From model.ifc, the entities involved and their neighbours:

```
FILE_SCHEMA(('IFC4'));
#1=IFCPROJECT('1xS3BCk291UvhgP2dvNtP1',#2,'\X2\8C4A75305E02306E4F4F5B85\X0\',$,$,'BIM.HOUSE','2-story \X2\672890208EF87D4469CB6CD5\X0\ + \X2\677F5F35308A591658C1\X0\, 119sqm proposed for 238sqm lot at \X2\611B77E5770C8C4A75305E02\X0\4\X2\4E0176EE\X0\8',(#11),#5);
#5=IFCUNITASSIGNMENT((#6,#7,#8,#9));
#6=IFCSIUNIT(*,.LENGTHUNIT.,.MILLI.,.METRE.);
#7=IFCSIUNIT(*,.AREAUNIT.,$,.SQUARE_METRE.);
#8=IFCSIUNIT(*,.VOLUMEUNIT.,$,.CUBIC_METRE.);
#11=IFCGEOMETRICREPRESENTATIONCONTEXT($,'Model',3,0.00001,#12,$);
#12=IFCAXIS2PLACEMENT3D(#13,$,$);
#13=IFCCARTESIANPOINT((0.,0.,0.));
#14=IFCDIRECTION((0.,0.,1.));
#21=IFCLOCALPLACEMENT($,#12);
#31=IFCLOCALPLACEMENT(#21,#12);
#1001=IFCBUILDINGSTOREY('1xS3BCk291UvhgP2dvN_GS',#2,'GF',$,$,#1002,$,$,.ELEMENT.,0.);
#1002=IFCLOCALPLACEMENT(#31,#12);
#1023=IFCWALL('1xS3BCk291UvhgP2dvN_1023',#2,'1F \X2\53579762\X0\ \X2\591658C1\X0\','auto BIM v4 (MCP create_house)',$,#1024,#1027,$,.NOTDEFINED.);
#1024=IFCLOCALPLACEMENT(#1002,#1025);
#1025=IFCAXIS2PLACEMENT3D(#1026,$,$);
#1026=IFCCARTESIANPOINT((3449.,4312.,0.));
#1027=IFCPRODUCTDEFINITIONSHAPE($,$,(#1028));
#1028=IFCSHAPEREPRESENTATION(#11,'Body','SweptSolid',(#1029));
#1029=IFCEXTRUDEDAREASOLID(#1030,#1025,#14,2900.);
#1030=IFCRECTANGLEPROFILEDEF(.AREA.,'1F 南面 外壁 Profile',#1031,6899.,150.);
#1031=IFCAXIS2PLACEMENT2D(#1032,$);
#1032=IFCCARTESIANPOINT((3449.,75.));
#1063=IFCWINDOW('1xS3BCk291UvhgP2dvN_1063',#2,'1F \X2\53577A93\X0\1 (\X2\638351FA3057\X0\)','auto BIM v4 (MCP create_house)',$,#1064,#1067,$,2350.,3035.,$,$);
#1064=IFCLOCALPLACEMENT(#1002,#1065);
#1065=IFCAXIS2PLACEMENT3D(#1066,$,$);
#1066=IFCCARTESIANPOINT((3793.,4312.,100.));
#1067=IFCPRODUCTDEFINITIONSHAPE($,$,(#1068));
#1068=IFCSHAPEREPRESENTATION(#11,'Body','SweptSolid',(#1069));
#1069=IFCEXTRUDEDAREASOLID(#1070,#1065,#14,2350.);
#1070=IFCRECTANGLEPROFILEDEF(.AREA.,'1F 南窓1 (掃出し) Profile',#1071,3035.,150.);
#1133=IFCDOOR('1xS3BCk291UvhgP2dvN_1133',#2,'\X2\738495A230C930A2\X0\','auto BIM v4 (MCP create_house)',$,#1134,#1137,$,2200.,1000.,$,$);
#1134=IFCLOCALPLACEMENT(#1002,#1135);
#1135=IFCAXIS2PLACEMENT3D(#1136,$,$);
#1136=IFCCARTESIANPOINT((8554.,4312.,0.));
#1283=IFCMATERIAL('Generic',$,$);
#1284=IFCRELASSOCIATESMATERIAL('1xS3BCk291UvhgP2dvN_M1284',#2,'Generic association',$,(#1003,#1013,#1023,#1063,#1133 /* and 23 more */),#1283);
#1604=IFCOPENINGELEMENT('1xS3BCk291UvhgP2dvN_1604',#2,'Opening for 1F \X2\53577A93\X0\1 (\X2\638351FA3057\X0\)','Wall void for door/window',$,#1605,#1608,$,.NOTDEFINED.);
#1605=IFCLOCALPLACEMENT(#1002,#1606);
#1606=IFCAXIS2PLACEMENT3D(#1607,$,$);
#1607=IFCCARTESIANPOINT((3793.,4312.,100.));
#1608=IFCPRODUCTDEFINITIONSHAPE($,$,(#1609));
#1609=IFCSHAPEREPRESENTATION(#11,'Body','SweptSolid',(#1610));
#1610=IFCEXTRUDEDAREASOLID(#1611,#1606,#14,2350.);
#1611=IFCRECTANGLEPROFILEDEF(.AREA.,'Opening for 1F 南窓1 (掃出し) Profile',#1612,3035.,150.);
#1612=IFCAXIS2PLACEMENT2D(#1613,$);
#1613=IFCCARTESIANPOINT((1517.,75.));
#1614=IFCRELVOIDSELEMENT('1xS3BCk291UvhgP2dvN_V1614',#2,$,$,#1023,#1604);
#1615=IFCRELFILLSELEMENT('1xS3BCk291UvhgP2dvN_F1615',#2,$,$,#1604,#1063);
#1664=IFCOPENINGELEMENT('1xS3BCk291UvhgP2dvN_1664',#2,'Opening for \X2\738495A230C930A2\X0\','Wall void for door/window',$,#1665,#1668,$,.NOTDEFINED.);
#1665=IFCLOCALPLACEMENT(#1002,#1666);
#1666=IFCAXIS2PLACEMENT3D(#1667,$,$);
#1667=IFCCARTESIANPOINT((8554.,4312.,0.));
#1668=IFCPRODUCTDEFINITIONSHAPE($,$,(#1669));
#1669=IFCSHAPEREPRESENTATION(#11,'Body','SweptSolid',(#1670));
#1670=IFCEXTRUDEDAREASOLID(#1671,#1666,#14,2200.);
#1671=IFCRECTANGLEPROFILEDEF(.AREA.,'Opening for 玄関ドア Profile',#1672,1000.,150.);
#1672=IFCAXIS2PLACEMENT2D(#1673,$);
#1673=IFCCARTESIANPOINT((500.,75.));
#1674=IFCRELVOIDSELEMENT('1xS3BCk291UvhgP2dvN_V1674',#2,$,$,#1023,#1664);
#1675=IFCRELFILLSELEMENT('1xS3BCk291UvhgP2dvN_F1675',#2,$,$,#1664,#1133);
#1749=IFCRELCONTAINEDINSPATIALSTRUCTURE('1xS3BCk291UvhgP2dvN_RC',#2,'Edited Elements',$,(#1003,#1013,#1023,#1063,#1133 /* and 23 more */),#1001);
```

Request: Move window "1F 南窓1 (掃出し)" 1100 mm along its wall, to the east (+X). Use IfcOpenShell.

```python
import ifcopenshell
import ifcopenshell.api.geometry
import ifcopenshell.util.placement
import ifcopenshell.util.unit

model = ifcopenshell.open("model.ifc")
unit_scale = ifcopenshell.util.unit.calculate_unit_scale(model)

window = model.by_id(1063)
opening = window.FillsVoids[0].RelatingOpeningElement
wall = opening.VoidsElements[0].RelatingBuildingElement

wall_matrix = ifcopenshell.util.placement.get_local_placement(wall.ObjectPlacement)
shift = wall_matrix[:3, 0] * 1.1 / unit_scale
before = ifcopenshell.util.placement.get_local_placement(window.ObjectPlacement)[:3, 3].copy()

# The window is not placed relative to its opening, so move both.
for product in (opening, window):
    matrix = ifcopenshell.util.placement.get_local_placement(product.ObjectPlacement)
    matrix[:3, 3] += shift
    ifcopenshell.api.geometry.edit_object_placement(model, product=product, matrix=matrix, is_si=False)

after = ifcopenshell.util.placement.get_local_placement(window.ObjectPlacement)[:3, 3]
print("window moved by", (after - before).round(3) + 0.0)

model.write("model_edited.ifc")
```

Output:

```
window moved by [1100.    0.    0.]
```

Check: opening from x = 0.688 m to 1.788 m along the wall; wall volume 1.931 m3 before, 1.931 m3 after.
